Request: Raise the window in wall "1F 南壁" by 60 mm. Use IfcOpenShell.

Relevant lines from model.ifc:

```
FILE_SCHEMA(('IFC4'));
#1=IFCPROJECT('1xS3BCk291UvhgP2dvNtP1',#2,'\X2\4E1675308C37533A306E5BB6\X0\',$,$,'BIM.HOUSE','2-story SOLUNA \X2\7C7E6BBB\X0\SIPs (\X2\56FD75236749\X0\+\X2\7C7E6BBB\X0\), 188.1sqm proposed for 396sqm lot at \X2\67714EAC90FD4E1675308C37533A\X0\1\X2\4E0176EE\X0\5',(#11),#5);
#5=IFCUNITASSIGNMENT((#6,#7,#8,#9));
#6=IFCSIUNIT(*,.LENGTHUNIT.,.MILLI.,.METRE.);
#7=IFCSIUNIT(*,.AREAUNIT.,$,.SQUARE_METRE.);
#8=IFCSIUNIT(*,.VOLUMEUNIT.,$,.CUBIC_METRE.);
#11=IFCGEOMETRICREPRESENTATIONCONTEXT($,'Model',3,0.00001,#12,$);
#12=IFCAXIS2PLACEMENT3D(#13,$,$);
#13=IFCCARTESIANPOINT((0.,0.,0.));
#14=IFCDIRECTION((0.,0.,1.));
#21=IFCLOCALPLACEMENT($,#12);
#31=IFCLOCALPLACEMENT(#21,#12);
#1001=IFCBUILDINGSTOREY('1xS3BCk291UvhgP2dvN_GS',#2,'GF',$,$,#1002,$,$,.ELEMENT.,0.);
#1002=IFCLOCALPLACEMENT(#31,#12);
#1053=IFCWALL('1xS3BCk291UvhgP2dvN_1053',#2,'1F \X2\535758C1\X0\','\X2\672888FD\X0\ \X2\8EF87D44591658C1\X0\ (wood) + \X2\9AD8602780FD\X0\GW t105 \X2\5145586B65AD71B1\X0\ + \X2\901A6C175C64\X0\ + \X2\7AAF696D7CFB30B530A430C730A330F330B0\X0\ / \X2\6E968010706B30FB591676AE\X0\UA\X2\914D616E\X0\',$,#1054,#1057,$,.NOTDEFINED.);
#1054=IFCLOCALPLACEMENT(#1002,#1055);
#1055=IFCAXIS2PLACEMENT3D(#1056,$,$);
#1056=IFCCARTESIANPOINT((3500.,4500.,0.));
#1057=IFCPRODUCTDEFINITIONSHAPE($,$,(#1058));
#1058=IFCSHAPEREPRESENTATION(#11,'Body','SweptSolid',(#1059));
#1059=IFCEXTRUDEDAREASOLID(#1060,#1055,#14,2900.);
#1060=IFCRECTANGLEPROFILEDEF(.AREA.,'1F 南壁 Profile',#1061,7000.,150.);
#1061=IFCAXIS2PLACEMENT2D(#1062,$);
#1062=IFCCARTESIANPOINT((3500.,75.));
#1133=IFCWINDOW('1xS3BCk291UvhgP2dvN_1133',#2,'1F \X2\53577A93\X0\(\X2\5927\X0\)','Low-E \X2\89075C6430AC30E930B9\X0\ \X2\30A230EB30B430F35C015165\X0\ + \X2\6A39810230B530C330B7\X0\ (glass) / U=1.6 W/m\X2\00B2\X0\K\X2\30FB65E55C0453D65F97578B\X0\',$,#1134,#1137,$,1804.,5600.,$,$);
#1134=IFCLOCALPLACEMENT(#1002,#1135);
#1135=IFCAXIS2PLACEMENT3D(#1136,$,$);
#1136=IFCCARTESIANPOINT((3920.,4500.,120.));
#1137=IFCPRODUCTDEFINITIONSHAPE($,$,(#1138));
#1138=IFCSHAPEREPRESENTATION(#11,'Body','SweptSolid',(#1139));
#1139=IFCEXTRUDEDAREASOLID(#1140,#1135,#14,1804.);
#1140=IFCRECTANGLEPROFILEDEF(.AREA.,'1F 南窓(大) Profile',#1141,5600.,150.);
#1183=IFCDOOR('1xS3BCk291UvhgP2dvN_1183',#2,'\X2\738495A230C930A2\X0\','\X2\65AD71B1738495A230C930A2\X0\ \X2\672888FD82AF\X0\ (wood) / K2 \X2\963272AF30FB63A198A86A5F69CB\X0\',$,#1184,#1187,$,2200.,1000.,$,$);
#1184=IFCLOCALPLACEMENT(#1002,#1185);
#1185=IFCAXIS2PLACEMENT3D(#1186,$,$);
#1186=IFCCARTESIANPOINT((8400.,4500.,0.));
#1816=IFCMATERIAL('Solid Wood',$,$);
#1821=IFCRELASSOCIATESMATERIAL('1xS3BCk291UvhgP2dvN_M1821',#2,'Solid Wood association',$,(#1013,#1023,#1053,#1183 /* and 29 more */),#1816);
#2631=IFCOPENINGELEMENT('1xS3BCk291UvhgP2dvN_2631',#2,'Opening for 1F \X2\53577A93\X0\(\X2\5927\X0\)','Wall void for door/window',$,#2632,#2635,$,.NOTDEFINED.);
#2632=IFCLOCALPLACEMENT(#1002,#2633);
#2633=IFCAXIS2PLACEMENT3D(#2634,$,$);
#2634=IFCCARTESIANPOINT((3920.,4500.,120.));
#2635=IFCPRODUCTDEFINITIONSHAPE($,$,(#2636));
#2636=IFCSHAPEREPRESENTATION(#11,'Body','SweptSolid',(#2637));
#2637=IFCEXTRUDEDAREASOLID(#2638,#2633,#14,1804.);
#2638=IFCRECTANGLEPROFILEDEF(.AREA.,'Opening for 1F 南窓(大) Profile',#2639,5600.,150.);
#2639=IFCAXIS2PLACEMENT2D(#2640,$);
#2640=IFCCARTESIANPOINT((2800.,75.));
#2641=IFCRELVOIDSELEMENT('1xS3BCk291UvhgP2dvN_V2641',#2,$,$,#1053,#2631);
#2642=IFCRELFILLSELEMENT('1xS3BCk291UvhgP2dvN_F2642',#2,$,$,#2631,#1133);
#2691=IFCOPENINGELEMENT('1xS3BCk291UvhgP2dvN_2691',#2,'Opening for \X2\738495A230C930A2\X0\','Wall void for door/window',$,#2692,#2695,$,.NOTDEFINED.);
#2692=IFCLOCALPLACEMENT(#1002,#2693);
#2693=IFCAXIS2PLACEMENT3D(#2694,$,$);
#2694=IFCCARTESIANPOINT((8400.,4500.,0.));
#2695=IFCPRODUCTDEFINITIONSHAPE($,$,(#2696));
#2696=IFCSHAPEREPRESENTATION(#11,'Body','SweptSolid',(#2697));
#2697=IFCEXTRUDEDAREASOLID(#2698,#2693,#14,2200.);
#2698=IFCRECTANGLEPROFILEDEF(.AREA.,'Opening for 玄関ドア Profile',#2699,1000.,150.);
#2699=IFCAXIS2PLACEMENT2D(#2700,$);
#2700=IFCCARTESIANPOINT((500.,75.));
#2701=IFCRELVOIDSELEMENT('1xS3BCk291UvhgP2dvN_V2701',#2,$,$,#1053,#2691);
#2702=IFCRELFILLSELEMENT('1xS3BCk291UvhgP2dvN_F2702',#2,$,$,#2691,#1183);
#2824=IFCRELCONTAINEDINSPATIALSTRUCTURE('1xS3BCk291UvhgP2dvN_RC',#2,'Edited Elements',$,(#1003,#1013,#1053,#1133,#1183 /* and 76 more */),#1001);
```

```python
import numpy as np
import ifcopenshell
import ifcopenshell.api.geometry
import ifcopenshell.util.placement
import ifcopenshell.util.unit

model = ifcopenshell.open("model.ifc")
unit_scale = ifcopenshell.util.unit.calculate_unit_scale(model)

window = model.by_guid("1xS3BCk291UvhgP2dvN_1133")
opening = window.FillsVoids[0].RelatingOpeningElement
dz = 0.06 / unit_scale

shift = np.array([0.0, 0.0, dz])
# The window is not placed relative to its opening, so move both.
for product in (opening, window):
    matrix = ifcopenshell.util.placement.get_local_placement(product.ObjectPlacement)
    matrix[:3, 3] += shift
    ifcopenshell.api.geometry.edit_object_placement(model, product=product, matrix=matrix, is_si=False)

print(f"moved by {dz * unit_scale:+.3f} m")

model.write("model_rev.ifc")
```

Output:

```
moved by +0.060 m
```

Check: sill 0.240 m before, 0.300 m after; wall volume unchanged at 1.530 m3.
